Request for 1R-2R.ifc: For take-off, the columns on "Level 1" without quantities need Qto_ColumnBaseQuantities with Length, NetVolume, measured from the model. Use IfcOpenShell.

First a look at what the model holds.

```python
import ifcopenshell
import ifcopenshell.util.element
import ifcopenshell.util.unit

model = ifcopenshell.open("1R-2R.ifc")
print(model.schema)
for unit_type in ("LENGTHUNIT", "AREAUNIT", "VOLUMEUNIT"):
    print(unit_type, ifcopenshell.util.unit.calculate_unit_scale(model, unit_type))
storey = next(s for s in model.by_type("IfcBuildingStorey") if s.Name == "Level 1")
columns = [e for e in ifcopenshell.util.element.get_decomposition(storey) if e.is_a("IfcColumn")]
for e in sorted(columns, key=lambda e: e.id()):
    print(e.id(), e.is_a(), e.Name, list(ifcopenshell.util.element.get_psets(e, qtos_only=True)), sep=" | ")
```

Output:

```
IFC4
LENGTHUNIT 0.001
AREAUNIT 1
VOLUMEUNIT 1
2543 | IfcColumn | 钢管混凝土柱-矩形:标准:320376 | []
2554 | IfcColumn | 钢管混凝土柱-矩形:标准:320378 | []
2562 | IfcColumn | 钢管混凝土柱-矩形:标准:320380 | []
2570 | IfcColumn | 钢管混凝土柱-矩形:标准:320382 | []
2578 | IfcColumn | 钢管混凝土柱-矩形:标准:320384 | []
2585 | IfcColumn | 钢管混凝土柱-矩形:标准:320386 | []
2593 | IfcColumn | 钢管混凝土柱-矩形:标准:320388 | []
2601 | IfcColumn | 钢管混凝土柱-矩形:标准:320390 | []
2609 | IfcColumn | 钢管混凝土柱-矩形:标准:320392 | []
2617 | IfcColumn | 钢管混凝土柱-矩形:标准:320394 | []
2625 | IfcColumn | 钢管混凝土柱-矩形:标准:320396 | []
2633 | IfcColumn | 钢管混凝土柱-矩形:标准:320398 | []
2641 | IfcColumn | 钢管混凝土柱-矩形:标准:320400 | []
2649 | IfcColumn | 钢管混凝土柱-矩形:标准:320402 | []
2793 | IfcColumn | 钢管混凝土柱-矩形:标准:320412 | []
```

```python
import ifcopenshell
import ifcopenshell.api.pset
import ifcopenshell.geom
import ifcopenshell.util.element
import ifcopenshell.util.shape
import ifcopenshell.util.unit

model = ifcopenshell.open("1R-2R.ifc")
unit_scale = ifcopenshell.util.unit.calculate_unit_scale(model)
volume_scale = ifcopenshell.util.unit.calculate_unit_scale(model, "VOLUMEUNIT")
settings = ifcopenshell.geom.settings()

storey = next(s for s in model.by_type("IfcBuildingStorey") if s.Name == "Level 1")
columns = [e for e in ifcopenshell.util.element.get_decomposition(storey) if e.is_a("IfcColumn")]

for e in sorted(columns, key=lambda e: e.id()):
    if ifcopenshell.util.element.get_psets(e, qtos_only=True, should_inherit=False):
        continue
    # Geometry comes back in metres, in the element's own axes.
    shape = ifcopenshell.geom.create_shape(settings, e)
    values = {
        "Length": ifcopenshell.util.shape.get_z(shape.geometry) / unit_scale,
        "NetVolume": ifcopenshell.util.shape.get_volume(shape.geometry) / volume_scale,
    }
    qto = ifcopenshell.api.pset.add_qto(model, product=e, name="Qto_ColumnBaseQuantities")
    ifcopenshell.api.pset.edit_qto(model, qto=qto, properties=values)
    print(e.id(), {k: round(v, 3) for k, v in values.items()})

model.write("1R-2R_edited.ifc")
```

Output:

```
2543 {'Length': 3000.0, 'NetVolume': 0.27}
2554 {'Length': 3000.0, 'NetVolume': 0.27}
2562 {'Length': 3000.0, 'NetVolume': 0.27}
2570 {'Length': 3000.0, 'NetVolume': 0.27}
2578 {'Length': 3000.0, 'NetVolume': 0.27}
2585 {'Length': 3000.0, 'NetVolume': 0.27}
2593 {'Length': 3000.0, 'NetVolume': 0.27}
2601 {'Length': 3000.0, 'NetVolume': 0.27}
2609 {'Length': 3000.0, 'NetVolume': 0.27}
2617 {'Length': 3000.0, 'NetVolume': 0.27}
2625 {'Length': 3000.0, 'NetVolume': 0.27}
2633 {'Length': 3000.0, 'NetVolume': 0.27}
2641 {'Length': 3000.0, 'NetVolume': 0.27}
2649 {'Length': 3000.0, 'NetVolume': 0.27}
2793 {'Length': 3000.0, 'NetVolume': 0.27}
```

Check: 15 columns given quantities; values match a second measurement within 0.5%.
